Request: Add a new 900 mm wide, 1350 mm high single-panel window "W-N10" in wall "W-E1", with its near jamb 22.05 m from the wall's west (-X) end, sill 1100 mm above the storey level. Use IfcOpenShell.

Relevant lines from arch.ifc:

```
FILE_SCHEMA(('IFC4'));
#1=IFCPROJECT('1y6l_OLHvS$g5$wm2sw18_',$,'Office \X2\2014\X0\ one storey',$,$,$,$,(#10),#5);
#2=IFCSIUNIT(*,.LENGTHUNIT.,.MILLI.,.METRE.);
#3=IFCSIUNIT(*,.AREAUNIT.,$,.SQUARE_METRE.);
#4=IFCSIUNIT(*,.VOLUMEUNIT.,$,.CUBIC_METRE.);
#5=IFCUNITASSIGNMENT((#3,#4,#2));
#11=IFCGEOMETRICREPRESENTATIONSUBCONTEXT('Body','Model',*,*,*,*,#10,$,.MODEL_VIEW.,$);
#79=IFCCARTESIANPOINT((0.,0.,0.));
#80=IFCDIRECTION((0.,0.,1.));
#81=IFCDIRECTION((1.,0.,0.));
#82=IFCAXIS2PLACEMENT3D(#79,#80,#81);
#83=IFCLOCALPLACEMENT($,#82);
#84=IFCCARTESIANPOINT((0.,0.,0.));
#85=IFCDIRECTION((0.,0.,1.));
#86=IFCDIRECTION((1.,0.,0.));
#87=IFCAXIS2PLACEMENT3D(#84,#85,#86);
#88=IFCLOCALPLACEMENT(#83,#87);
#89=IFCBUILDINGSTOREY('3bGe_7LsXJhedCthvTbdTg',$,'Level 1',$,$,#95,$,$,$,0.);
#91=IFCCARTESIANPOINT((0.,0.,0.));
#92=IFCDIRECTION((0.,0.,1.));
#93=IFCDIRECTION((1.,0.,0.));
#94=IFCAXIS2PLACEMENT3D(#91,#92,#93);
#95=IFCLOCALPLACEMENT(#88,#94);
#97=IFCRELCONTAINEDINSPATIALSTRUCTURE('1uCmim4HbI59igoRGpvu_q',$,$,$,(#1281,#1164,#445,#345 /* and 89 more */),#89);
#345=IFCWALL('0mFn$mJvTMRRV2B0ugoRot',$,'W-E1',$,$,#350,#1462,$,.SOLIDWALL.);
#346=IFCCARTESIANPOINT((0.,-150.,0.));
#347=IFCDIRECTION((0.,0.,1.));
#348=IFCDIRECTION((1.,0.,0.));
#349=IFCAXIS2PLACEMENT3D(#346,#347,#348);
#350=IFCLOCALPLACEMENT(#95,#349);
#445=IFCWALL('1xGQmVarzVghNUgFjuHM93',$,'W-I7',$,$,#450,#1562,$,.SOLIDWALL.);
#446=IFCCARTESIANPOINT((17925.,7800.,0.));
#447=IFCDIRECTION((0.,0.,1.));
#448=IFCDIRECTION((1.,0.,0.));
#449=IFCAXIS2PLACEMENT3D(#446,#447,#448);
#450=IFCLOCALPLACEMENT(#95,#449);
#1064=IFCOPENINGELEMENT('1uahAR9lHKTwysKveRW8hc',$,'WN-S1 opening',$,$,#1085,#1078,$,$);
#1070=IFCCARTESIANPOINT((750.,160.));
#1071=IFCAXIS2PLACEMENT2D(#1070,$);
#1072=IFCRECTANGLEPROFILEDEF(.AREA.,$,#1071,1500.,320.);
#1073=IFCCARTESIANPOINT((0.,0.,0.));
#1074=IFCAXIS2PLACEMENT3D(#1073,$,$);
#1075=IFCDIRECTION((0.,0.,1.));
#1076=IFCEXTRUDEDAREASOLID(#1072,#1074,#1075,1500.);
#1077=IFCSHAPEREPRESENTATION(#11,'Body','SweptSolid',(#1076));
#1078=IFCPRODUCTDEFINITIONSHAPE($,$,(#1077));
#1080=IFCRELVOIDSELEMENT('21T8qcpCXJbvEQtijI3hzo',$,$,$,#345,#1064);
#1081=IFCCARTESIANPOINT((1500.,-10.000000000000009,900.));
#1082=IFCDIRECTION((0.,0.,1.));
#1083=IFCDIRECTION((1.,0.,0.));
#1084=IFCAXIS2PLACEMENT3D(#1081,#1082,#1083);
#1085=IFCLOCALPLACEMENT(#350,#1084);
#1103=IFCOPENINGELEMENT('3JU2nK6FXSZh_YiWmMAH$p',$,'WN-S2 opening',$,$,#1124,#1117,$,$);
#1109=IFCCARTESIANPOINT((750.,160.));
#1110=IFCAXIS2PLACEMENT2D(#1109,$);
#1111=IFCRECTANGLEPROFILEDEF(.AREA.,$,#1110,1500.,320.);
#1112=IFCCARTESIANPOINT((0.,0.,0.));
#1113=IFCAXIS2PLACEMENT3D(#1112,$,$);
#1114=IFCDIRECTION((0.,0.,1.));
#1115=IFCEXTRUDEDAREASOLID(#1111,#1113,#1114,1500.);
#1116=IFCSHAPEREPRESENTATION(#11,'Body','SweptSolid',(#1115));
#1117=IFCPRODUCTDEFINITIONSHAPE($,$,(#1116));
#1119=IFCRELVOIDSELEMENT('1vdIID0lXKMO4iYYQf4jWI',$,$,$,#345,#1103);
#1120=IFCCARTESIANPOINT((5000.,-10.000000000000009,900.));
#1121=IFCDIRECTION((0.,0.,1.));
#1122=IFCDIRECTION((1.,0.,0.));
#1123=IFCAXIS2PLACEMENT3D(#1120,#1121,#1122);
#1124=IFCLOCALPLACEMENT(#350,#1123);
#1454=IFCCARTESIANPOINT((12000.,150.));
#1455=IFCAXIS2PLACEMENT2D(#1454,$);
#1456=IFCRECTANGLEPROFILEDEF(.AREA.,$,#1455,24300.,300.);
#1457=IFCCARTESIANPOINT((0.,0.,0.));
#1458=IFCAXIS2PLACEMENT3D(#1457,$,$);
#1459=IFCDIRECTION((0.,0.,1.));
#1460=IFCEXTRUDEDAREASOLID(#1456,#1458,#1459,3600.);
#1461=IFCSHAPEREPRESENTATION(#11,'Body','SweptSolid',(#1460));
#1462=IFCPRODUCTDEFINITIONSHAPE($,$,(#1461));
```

```python
import numpy as np
import ifcopenshell
import ifcopenshell.api.feature
import ifcopenshell.api.geometry
import ifcopenshell.api.root
import ifcopenshell.api.spatial
import ifcopenshell.geom
import ifcopenshell.util.element
import ifcopenshell.util.placement
import ifcopenshell.util.representation
import ifcopenshell.util.shape
import ifcopenshell.util.unit

model = ifcopenshell.open("arch.ifc")
unit_scale = ifcopenshell.util.unit.calculate_unit_scale(model)
settings = ifcopenshell.geom.settings()


def volume(element):
    """Net volume in cubic metres, openings subtracted."""
    shape = ifcopenshell.geom.create_shape(settings, element)
    return ifcopenshell.util.shape.get_volume(shape.geometry)


wall = model.by_guid("0mFn$mJvTMRRV2B0ugoRot")
storey = ifcopenshell.util.element.get_container(wall, ifc_class="IfcBuildingStorey")
context = ifcopenshell.util.representation.get_context(model, "Model", "Body", "MODEL_VIEW")
before = volume(wall)

width, height, from_end, sill = 0.9, 1.35, 22.05, 1.1  # metres

# The wall runs along its own X axis, and the end named is its -X end.
wall_shape = ifcopenshell.geom.create_shape(settings, wall)
x, y, z = ifcopenshell.util.shape.get_vertices(wall_shape.geometry).T
start = x.min() + from_end
face, thickness = float(y.min()), float(y.max() - y.min())
wall_matrix = ifcopenshell.util.placement.get_local_placement(wall.ObjectPlacement)
level = ifcopenshell.util.placement.get_local_placement(storey.ObjectPlacement)[2, 3]


def in_wall(x, y):
    """Placement at x, y metres in the wall's axes, at sill height."""
    matrix = wall_matrix.copy()
    matrix[:, 3] = wall_matrix @ np.array([x / unit_scale, y / unit_scale, 0.0, 1.0])
    matrix[2, 3] = level + sill / unit_scale
    return matrix


# Opening: a box that overshoots both wall faces by 50 mm.
opening = ifcopenshell.api.root.create_entity(model, ifc_class="IfcOpeningElement", predefined_type="OPENING")
box = ifcopenshell.api.geometry.add_wall_representation(
    model, context=context, length=width, height=height, thickness=thickness + 0.1
)
ifcopenshell.api.geometry.assign_representation(model, product=opening, representation=box)
ifcopenshell.api.geometry.edit_object_placement(model, product=opening, matrix=in_wall(start, face - 0.05), is_si=False)
ifcopenshell.api.feature.add_feature(model, feature=opening, element=wall)

window = ifcopenshell.api.root.create_entity(model, ifc_class="IfcWindow", name="W-N10", predefined_type="WINDOW")
window.OverallWidth, window.OverallHeight = width / unit_scale, height / unit_scale
window.PartitioningType = "SINGLE_PANEL"
body = ifcopenshell.api.geometry.add_window_representation(
    model,
    context=context,
    overall_width=window.OverallWidth,
    overall_height=window.OverallHeight,
    partition_type="SINGLE_PANEL",
)
ifcopenshell.api.geometry.assign_representation(model, product=window, representation=body)
ifcopenshell.api.spatial.assign_container(model, products=[window], relating_structure=storey)
ifcopenshell.api.feature.add_filling(model, opening=opening, element=window)

# Centre the window in the wall's thickness.
ifcopenshell.api.geometry.edit_object_placement(model, product=window, matrix=in_wall(start, face), is_si=False)
window_shape = ifcopenshell.geom.create_shape(settings, window)
depth = ifcopenshell.util.shape.get_vertices(window_shape.geometry)[:, 1]
offset = face + thickness / 2 - (depth.min() + depth.max()) / 2
ifcopenshell.api.geometry.edit_object_placement(model, product=window, matrix=in_wall(start, offset), is_si=False)

after = volume(wall)

print(f"wall volume {before:.3f} -> {after:.3f} m3")

model.write("arch_v2.ifc")
```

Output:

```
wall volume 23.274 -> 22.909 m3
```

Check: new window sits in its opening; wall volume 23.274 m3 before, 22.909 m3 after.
